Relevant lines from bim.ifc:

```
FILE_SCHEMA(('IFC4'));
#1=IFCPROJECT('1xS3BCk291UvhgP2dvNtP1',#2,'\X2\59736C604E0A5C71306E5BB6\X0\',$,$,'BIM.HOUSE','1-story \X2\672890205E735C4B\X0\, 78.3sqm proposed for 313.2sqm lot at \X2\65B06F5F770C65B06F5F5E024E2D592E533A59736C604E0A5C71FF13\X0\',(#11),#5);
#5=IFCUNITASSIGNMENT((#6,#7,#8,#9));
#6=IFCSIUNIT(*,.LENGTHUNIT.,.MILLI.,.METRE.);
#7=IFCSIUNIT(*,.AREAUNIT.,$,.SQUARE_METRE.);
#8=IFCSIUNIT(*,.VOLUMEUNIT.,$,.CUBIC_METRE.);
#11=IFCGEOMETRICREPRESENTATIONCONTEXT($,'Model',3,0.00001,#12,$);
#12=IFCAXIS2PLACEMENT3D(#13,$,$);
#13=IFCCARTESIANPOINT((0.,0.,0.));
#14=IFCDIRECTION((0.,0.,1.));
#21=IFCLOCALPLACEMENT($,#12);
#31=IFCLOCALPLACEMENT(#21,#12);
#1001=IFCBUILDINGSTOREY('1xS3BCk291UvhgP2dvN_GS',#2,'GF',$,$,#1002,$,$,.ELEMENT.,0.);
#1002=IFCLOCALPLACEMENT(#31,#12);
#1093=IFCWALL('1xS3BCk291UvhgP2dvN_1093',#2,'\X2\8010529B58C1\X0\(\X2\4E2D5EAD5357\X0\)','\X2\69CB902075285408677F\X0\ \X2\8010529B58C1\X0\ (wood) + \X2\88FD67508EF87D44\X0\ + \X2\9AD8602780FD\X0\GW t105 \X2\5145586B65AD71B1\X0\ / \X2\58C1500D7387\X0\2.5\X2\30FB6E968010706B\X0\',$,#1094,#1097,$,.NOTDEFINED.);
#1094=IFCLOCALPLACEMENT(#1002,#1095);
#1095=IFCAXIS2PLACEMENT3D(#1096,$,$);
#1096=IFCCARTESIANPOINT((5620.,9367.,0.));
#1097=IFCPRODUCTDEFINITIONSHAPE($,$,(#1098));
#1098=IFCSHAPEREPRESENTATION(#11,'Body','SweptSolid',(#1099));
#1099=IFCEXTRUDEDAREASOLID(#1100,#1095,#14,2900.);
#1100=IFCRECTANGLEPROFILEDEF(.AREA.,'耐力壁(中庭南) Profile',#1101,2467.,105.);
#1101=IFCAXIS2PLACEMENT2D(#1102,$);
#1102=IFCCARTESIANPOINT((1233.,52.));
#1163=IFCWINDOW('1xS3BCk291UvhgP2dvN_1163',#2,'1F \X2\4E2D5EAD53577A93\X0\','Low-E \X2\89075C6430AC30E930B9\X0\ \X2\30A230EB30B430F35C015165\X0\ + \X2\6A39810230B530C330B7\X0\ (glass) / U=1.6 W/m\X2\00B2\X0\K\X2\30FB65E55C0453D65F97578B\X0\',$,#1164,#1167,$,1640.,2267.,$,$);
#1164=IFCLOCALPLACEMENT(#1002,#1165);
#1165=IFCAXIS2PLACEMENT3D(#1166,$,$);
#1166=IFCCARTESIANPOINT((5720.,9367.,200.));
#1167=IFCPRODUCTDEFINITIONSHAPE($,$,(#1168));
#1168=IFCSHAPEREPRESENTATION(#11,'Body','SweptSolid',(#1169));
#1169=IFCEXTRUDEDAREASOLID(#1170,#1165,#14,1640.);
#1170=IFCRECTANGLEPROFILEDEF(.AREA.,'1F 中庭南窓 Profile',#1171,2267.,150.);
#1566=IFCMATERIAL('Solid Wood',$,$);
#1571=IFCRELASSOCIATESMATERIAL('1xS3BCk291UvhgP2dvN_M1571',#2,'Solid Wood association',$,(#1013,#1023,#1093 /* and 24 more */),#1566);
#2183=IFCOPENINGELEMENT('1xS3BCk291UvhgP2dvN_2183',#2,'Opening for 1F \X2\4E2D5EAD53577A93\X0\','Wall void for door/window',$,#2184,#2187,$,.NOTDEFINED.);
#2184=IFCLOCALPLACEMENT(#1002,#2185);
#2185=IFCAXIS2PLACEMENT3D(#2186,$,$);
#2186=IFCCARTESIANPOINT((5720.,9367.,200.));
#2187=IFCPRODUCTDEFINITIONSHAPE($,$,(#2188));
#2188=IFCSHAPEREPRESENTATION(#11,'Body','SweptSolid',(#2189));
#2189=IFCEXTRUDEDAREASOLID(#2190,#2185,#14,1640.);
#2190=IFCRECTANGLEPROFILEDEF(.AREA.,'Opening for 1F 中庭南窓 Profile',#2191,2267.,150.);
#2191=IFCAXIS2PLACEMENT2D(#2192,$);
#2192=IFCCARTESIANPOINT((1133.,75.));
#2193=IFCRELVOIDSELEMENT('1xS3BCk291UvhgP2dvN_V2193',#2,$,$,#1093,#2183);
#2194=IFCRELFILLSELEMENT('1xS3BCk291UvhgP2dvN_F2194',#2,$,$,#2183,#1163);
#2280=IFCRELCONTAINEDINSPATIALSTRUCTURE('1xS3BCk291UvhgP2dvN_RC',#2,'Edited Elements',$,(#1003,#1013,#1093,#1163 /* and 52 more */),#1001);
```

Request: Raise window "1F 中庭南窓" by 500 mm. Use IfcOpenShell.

```python
import numpy as np
import ifcopenshell
import ifcopenshell.api.geometry
import ifcopenshell.util.placement
import ifcopenshell.util.unit

model = ifcopenshell.open("bim.ifc")
unit_scale = ifcopenshell.util.unit.calculate_unit_scale(model)

window = model.by_id(1163)
opening = window.FillsVoids[0].RelatingOpeningElement
dz = 0.5 / unit_scale

shift = np.array([0.0, 0.0, dz])
# The window is not placed relative to its opening, so move both.
for product in (opening, window):
    matrix = ifcopenshell.util.placement.get_local_placement(product.ObjectPlacement)
    matrix[:3, 3] += shift
    ifcopenshell.api.geometry.edit_object_placement(model, product=product, matrix=matrix, is_si=False)

print(f"moved by {dz * unit_scale:+.3f} m")

model.write("bim_updated.ifc")
```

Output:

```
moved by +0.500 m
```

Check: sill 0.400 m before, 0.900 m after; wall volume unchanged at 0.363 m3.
